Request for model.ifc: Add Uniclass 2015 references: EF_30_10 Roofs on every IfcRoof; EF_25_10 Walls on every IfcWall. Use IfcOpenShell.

First a look at what the model holds.

```python
import ifcopenshell

model = ifcopenshell.open("model.ifc")
print(model.schema)
print("classifications:", [c.Name for c in model.by_type("IfcClassification")])
for ifc_class in ("IfcDoor", "IfcRoof", "IfcStair", "IfcWall", "IfcWindow"):
    print(ifc_class, len(model.by_type(ifc_class)))
```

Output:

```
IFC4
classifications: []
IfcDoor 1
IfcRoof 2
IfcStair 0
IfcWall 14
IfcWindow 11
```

```python
import ifcopenshell
import ifcopenshell.api.classification

model = ifcopenshell.open("model.ifc")

system = ifcopenshell.api.classification.add_classification(model, classification="Uniclass 2015")

codes = {
    "IfcRoof": ("EF_30_10", "Roofs"),
    "IfcWall": ("EF_25_10", "Walls"),
}
for ifc_class, (code, name) in codes.items():
    products = model.by_type(ifc_class)
    ifcopenshell.api.classification.add_reference(
        model, products=products, classification=system, identification=code, name=name
    )
    print(code, len(products))

model.write("model_rev.ifc")
```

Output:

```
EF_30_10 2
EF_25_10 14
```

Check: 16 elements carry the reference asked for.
